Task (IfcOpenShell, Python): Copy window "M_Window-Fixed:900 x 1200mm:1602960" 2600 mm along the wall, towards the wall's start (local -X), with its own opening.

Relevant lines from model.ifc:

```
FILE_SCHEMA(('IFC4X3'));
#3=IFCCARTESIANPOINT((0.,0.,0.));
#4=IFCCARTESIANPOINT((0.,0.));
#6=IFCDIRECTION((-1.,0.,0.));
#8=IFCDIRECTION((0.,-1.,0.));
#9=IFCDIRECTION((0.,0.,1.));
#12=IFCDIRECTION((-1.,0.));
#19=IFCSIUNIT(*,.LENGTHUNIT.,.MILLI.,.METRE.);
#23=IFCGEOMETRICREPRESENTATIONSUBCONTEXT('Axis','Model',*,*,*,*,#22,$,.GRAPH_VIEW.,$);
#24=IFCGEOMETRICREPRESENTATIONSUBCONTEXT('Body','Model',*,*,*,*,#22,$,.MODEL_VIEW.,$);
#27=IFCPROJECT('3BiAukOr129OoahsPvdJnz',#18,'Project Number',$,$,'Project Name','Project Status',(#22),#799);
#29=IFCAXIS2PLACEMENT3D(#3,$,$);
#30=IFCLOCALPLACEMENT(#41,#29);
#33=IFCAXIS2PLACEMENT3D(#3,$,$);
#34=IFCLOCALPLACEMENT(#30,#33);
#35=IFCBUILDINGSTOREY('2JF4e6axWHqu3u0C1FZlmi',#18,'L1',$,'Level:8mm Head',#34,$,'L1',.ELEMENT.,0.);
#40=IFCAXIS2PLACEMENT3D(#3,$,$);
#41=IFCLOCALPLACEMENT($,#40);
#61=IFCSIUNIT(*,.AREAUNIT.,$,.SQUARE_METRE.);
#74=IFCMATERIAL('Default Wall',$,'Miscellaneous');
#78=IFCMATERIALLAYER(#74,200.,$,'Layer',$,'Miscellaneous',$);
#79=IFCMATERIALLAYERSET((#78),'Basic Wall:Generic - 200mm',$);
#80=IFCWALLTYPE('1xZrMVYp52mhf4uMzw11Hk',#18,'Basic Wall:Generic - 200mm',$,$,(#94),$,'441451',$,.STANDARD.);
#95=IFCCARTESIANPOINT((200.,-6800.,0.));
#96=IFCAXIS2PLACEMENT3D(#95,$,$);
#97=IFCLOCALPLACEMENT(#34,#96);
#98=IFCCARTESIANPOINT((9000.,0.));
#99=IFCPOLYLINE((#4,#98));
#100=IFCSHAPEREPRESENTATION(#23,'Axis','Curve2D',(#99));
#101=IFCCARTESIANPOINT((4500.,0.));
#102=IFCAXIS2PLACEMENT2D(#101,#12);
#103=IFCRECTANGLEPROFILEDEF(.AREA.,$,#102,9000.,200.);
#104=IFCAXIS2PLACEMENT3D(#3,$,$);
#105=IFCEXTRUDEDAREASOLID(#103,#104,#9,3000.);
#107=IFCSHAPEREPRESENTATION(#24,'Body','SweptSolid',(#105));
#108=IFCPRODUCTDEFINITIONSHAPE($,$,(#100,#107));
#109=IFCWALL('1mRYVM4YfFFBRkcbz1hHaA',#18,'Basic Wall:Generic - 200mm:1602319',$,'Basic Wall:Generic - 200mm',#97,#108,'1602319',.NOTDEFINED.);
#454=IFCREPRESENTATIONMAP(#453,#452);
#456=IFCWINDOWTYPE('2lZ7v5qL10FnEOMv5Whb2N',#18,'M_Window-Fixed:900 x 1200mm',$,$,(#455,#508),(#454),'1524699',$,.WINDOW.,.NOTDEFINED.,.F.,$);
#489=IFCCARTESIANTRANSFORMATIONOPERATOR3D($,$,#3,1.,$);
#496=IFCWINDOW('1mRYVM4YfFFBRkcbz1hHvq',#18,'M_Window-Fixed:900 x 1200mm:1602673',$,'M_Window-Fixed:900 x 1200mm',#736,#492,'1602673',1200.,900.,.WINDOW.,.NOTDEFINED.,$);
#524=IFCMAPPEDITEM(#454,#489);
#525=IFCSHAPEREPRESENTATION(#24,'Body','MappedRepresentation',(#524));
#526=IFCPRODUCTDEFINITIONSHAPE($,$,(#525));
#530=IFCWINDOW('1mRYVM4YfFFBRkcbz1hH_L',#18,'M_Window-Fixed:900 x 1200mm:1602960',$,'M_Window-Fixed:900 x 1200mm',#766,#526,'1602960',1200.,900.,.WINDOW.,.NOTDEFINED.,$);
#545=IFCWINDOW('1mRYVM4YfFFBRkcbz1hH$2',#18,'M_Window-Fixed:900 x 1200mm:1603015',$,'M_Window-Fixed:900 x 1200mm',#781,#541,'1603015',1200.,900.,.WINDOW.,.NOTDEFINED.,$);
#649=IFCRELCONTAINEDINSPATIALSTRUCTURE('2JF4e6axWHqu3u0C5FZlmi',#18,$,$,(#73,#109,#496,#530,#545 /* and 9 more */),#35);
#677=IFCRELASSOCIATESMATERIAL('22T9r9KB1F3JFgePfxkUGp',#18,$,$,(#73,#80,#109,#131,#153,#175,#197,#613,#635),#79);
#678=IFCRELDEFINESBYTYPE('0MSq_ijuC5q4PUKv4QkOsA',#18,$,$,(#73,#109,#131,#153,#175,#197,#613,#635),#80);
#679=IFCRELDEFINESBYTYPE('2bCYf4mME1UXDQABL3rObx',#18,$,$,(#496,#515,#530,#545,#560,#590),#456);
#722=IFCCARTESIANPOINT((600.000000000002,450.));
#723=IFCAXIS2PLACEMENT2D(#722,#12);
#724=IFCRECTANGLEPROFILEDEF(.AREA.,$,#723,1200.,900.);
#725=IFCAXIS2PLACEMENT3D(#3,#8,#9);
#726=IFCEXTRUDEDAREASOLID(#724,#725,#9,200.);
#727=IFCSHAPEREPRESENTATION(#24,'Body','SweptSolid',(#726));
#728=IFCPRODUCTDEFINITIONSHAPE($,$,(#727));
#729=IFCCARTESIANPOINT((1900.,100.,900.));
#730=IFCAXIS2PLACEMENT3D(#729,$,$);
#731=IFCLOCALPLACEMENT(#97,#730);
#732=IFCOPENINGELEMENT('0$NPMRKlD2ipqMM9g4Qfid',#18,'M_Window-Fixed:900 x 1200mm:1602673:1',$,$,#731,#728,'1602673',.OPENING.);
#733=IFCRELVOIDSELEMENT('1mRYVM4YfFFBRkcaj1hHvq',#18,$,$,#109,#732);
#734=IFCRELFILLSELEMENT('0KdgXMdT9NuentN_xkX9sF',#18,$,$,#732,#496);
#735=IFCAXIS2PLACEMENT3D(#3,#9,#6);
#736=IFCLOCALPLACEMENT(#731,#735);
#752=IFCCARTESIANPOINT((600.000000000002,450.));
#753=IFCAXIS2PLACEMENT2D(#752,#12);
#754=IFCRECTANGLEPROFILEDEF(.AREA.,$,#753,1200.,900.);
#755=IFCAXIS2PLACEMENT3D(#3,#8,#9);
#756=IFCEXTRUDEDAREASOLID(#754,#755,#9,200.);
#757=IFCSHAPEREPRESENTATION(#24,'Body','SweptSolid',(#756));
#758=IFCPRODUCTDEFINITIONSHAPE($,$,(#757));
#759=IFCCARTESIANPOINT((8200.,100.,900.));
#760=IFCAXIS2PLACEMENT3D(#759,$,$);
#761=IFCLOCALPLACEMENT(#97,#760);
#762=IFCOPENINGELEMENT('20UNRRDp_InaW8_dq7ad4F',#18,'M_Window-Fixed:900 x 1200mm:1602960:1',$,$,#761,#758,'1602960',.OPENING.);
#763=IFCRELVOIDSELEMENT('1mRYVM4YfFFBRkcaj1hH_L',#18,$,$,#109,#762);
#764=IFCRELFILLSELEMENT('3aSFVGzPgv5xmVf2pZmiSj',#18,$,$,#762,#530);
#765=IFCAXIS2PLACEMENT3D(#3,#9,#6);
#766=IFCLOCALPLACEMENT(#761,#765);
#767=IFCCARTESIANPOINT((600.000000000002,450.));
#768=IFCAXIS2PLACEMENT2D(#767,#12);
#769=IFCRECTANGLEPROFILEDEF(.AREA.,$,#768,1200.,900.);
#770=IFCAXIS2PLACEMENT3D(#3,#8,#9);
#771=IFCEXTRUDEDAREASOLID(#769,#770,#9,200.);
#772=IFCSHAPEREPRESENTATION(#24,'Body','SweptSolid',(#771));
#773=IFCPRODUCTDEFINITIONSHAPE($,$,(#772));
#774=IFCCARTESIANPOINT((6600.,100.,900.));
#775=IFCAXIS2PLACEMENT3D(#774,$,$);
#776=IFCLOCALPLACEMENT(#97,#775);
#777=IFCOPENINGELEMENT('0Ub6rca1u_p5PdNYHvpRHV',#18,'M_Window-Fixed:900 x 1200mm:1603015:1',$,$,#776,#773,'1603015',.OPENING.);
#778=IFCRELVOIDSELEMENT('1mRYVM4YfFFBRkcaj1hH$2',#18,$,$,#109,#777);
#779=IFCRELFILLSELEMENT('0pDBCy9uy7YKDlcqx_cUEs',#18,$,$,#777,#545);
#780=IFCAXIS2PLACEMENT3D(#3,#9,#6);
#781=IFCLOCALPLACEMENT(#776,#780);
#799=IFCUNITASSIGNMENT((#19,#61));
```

```python
import ifcopenshell
import ifcopenshell.api.feature
import ifcopenshell.api.geometry
import ifcopenshell.api.root
import ifcopenshell.geom
import ifcopenshell.util.element
import ifcopenshell.util.placement
import ifcopenshell.util.shape
import ifcopenshell.util.unit

model = ifcopenshell.open("model.ifc")
unit_scale = ifcopenshell.util.unit.calculate_unit_scale(model)
settings = ifcopenshell.geom.settings()


def volume(element):
    """Net volume in cubic metres, openings subtracted."""
    shape = ifcopenshell.geom.create_shape(settings, element)
    return ifcopenshell.util.shape.get_volume(shape.geometry)


def reuse_history(source, copy):
    """copy_class also copies each property set's owner history, people and application; keep the originals."""
    for rel in copy.IsDefinedBy:
        if rel.is_a("IfcRelDefinesByProperties") and (history := rel.RelatingPropertyDefinition.OwnerHistory):
            rel.RelatingPropertyDefinition.OwnerHistory = source.OwnerHistory
            ifcopenshell.util.element.remove_deep2(model, history)


window = model.by_guid("1mRYVM4YfFFBRkcbz1hH_L")
opening = window.FillsVoids[0].RelatingOpeningElement
wall = opening.VoidsElements[0].RelatingBuildingElement
before = volume(wall)
shift = ifcopenshell.util.placement.get_local_placement(wall.ObjectPlacement)[:3, 0] * -2.6 / unit_scale

# copy_class copies the void relationship, type, container and properties, but no geometry.
new_opening = ifcopenshell.api.root.copy_class(model, product=opening)
new_opening.Representation = ifcopenshell.util.element.copy_deep(
    model, opening.Representation, exclude=["IfcGeometricRepresentationContext", "IfcRepresentationMap"]
)
new_opening.Name = "M_Window-Fixed:900 x 1200mm"
new_opening.Tag = None
new_window = ifcopenshell.api.root.copy_class(model, product=window)
new_window.Representation = ifcopenshell.util.element.copy_deep(
    model, window.Representation, exclude=["IfcGeometricRepresentationContext", "IfcRepresentationMap"]
)
new_window.Name = "M_Window-Fixed:900 x 1200mm"
new_window.Tag = None
reuse_history(window, new_window)
ifcopenshell.api.feature.add_filling(model, opening=new_opening, element=new_window)

for old, new in ((opening, new_opening), (window, new_window)):
    matrix = ifcopenshell.util.placement.get_local_placement(old.ObjectPlacement)
    matrix[:3, 3] += shift
    ifcopenshell.api.geometry.edit_object_placement(model, product=new, matrix=matrix, is_si=False)

after = volume(wall)

print(f"wall volume {before:.3f} -> {after:.3f} m3")

model.write("model_v2.ifc")
```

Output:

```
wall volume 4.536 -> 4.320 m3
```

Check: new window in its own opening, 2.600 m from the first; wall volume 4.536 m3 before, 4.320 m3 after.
